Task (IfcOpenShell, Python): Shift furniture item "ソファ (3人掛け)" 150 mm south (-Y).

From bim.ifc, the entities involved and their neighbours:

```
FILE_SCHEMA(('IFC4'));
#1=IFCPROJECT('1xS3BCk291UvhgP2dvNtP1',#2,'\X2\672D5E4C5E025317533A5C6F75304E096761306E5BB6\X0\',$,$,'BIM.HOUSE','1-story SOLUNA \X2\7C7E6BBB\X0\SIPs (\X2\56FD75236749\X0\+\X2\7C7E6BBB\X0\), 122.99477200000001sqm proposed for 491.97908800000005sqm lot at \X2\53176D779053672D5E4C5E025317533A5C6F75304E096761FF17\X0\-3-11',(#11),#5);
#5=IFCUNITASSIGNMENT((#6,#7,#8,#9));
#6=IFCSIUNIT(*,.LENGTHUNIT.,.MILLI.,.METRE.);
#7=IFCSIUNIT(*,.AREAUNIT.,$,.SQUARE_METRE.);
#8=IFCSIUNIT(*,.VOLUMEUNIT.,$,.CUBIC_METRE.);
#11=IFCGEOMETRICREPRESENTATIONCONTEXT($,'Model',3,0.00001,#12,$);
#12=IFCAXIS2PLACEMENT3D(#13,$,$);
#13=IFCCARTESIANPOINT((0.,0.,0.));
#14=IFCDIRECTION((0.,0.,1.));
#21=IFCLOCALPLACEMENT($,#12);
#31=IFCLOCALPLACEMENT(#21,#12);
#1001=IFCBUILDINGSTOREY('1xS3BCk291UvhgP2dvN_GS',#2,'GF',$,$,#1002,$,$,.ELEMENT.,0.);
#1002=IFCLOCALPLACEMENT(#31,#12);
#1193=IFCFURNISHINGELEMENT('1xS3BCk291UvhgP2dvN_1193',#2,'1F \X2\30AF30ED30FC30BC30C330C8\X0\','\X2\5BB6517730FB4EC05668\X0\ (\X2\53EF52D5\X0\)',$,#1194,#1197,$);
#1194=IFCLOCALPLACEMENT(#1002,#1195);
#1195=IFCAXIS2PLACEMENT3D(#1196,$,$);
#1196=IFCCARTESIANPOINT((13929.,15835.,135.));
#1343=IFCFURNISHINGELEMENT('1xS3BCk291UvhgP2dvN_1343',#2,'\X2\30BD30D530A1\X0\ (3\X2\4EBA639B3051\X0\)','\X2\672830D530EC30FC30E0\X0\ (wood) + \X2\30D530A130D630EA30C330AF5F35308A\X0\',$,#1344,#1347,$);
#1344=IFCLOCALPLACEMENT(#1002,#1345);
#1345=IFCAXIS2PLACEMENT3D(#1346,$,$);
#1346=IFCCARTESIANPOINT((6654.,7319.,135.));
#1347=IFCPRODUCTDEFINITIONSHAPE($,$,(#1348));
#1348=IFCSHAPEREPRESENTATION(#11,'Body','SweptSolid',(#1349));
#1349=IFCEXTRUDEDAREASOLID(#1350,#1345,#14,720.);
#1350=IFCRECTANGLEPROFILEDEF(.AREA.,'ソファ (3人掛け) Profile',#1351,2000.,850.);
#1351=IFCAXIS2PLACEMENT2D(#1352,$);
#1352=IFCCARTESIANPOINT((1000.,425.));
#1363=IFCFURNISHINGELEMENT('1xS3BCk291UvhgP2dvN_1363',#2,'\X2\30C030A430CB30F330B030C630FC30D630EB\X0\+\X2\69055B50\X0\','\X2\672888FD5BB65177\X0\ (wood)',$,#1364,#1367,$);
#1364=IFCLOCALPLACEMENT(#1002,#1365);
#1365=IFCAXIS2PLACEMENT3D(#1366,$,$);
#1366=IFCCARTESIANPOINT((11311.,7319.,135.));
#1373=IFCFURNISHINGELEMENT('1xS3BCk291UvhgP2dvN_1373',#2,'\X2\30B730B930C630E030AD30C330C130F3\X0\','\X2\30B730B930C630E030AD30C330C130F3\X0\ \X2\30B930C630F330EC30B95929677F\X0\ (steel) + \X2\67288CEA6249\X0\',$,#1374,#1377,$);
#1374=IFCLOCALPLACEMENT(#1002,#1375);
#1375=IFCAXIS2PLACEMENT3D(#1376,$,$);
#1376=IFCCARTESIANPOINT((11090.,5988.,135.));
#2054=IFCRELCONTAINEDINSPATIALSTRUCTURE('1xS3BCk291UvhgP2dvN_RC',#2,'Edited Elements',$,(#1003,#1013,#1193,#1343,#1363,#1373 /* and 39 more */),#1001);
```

```python
import ifcopenshell
import ifcopenshell.api.geometry
import ifcopenshell.util.placement

model = ifcopenshell.open("bim.ifc")

item = model.by_guid("1xS3BCk291UvhgP2dvN_1343")
matrix = ifcopenshell.util.placement.get_local_placement(item.ObjectPlacement)
matrix[1, 3] -= 150.0
ifcopenshell.api.geometry.edit_object_placement(model, product=item, matrix=matrix, is_si=False)

print(ifcopenshell.util.placement.get_local_placement(item.ObjectPlacement).round(3) + 0.0)

model.write("bim_v2.ifc")
```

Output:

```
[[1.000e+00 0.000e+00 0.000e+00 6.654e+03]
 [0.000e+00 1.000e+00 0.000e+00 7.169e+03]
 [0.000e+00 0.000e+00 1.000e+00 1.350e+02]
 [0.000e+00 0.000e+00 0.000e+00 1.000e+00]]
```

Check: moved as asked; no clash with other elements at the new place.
